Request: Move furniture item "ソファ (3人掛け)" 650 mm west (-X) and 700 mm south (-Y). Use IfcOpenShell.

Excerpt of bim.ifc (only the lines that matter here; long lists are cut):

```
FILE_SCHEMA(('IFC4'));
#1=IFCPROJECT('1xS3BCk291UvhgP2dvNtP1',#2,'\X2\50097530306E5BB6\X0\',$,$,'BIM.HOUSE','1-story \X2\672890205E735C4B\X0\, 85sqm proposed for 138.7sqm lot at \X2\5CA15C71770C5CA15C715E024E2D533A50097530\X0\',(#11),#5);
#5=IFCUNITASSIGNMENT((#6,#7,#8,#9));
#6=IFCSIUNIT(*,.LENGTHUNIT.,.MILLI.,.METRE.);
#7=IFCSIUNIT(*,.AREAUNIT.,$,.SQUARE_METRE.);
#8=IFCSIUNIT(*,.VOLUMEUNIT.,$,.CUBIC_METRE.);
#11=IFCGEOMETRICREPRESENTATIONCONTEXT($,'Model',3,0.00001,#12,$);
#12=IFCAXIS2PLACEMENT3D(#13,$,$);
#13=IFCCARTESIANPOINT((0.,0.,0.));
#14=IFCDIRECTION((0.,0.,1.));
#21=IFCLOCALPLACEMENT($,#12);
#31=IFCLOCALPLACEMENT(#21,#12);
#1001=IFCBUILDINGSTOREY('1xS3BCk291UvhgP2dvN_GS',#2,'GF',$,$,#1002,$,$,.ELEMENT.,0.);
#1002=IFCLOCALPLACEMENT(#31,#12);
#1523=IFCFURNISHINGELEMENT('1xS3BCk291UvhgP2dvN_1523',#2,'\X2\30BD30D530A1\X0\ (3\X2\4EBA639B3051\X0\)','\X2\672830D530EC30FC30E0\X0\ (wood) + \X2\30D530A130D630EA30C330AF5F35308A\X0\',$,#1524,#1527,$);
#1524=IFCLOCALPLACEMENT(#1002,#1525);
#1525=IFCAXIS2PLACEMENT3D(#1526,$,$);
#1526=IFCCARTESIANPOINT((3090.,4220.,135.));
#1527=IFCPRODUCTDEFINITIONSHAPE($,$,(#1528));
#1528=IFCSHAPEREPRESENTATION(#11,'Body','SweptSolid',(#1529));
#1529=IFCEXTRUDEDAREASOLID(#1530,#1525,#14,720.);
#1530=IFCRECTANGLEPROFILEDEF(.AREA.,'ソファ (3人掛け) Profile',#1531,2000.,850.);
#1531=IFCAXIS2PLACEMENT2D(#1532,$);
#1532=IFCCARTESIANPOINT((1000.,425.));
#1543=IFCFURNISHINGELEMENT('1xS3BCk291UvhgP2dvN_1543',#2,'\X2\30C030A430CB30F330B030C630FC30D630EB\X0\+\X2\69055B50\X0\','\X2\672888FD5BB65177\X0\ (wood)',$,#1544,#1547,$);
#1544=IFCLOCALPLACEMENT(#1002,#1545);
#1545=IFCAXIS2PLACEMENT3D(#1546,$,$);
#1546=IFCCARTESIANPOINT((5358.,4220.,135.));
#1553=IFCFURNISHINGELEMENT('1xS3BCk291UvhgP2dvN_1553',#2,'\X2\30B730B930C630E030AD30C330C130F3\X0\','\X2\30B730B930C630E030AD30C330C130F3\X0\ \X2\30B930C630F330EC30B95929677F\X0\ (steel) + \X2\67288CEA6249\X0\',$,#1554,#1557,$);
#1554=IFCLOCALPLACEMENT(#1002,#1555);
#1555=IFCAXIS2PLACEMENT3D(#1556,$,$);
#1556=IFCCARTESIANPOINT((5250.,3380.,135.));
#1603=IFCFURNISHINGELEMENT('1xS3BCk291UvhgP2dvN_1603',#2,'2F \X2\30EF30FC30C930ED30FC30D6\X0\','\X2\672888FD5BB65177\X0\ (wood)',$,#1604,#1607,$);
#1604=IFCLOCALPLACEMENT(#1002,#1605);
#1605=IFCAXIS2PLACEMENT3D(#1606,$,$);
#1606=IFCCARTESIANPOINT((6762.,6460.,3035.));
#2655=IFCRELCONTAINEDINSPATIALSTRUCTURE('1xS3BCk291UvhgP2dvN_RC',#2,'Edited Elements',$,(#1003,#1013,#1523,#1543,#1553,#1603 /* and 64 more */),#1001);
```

```python
import ifcopenshell
import ifcopenshell.api.geometry
import ifcopenshell.util.placement

model = ifcopenshell.open("bim.ifc")

item = model.by_guid("1xS3BCk291UvhgP2dvN_1523")
matrix = ifcopenshell.util.placement.get_local_placement(item.ObjectPlacement)
matrix[0, 3] -= 650.0
matrix[1, 3] -= 700.0
ifcopenshell.api.geometry.edit_object_placement(model, product=item, matrix=matrix, is_si=False)

print(ifcopenshell.util.placement.get_local_placement(item.ObjectPlacement).round(3) + 0.0)

model.write("bim_v2.ifc")
```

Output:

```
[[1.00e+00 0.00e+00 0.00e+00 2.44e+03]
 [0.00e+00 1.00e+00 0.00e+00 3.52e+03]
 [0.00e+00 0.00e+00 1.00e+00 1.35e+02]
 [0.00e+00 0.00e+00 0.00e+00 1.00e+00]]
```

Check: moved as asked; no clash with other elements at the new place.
